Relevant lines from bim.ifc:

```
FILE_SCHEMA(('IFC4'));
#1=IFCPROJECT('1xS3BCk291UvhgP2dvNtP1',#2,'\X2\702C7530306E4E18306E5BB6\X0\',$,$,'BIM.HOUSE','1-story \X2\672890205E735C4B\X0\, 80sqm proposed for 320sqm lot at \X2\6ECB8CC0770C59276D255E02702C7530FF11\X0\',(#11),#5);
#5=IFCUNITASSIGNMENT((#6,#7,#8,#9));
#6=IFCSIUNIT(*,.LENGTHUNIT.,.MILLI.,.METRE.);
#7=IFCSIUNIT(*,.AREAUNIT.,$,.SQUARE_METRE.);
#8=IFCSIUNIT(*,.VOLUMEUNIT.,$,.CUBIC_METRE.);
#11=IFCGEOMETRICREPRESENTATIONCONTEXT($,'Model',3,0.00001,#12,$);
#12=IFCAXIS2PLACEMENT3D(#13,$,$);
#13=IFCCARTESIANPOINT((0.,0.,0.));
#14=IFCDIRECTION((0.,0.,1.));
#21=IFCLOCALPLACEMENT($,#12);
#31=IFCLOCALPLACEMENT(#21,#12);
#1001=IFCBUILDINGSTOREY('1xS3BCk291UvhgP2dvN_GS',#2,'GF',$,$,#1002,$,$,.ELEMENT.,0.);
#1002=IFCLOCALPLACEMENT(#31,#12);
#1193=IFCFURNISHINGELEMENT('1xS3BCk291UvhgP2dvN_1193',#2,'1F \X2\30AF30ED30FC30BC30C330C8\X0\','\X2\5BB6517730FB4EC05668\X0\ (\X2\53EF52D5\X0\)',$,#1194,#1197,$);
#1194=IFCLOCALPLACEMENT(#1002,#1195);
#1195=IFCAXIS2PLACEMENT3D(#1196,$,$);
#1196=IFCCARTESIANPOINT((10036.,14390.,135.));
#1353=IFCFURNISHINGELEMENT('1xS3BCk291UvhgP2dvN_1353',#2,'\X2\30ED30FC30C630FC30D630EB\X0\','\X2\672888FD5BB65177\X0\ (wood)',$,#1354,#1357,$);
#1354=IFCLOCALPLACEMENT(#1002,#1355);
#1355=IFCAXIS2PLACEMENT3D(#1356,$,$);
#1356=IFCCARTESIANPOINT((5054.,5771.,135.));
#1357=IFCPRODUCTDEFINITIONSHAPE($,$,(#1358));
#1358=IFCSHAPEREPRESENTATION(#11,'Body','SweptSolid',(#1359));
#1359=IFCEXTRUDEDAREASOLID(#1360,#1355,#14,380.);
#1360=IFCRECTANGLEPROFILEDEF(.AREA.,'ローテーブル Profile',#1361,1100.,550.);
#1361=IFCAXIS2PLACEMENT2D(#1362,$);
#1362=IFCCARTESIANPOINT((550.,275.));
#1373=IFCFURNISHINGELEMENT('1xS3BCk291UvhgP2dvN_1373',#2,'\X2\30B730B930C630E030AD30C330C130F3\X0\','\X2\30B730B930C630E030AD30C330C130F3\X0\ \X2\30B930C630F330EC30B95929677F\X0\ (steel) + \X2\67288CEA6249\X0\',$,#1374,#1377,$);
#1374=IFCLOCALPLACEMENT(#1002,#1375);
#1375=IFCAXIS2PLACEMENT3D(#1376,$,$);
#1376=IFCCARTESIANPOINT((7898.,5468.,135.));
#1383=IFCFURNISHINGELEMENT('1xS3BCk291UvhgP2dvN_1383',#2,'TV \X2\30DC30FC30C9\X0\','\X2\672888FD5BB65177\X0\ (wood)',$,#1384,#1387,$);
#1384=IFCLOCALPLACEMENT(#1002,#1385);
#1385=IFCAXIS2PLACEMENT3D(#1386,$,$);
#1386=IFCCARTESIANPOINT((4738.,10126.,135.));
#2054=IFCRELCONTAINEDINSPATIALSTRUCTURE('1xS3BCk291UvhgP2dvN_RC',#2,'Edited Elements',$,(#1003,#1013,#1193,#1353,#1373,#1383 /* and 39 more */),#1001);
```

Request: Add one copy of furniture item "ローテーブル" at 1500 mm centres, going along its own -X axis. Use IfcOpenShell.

```python
import ifcopenshell
import ifcopenshell.api.geometry
import ifcopenshell.api.root
import ifcopenshell.util.element
import ifcopenshell.util.placement

model = ifcopenshell.open("bim.ifc")


def reuse_history(source, copy):
    """copy_class also copies each property set's owner history, people and application; keep the originals."""
    for rel in copy.IsDefinedBy:
        if rel.is_a("IfcRelDefinesByProperties") and (history := rel.RelatingPropertyDefinition.OwnerHistory):
            rel.RelatingPropertyDefinition.OwnerHistory = source.OwnerHistory
            ifcopenshell.util.element.remove_deep2(model, history)


source = model.by_guid("1xS3BCk291UvhgP2dvN_1353")
base = ifcopenshell.util.placement.get_local_placement(source.ObjectPlacement)
step = -base[:3, 0] * 1500.0

for i in range(1, 2):
    copy = ifcopenshell.api.root.copy_class(model, product=source)
    copy.Representation = ifcopenshell.util.element.copy_deep(
        model, source.Representation, exclude=["IfcGeometricRepresentationContext", "IfcRepresentationMap"]
    )
    reuse_history(source, copy)
    matrix = base.copy()
    matrix[:3, 3] += i * step
    print("added at", matrix[:3, 3].round(3) + 0.0)
    ifcopenshell.api.geometry.edit_object_placement(model, product=copy, matrix=matrix, is_si=False)

model.write("bim_updated.ifc")
```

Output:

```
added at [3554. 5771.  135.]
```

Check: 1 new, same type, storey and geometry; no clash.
